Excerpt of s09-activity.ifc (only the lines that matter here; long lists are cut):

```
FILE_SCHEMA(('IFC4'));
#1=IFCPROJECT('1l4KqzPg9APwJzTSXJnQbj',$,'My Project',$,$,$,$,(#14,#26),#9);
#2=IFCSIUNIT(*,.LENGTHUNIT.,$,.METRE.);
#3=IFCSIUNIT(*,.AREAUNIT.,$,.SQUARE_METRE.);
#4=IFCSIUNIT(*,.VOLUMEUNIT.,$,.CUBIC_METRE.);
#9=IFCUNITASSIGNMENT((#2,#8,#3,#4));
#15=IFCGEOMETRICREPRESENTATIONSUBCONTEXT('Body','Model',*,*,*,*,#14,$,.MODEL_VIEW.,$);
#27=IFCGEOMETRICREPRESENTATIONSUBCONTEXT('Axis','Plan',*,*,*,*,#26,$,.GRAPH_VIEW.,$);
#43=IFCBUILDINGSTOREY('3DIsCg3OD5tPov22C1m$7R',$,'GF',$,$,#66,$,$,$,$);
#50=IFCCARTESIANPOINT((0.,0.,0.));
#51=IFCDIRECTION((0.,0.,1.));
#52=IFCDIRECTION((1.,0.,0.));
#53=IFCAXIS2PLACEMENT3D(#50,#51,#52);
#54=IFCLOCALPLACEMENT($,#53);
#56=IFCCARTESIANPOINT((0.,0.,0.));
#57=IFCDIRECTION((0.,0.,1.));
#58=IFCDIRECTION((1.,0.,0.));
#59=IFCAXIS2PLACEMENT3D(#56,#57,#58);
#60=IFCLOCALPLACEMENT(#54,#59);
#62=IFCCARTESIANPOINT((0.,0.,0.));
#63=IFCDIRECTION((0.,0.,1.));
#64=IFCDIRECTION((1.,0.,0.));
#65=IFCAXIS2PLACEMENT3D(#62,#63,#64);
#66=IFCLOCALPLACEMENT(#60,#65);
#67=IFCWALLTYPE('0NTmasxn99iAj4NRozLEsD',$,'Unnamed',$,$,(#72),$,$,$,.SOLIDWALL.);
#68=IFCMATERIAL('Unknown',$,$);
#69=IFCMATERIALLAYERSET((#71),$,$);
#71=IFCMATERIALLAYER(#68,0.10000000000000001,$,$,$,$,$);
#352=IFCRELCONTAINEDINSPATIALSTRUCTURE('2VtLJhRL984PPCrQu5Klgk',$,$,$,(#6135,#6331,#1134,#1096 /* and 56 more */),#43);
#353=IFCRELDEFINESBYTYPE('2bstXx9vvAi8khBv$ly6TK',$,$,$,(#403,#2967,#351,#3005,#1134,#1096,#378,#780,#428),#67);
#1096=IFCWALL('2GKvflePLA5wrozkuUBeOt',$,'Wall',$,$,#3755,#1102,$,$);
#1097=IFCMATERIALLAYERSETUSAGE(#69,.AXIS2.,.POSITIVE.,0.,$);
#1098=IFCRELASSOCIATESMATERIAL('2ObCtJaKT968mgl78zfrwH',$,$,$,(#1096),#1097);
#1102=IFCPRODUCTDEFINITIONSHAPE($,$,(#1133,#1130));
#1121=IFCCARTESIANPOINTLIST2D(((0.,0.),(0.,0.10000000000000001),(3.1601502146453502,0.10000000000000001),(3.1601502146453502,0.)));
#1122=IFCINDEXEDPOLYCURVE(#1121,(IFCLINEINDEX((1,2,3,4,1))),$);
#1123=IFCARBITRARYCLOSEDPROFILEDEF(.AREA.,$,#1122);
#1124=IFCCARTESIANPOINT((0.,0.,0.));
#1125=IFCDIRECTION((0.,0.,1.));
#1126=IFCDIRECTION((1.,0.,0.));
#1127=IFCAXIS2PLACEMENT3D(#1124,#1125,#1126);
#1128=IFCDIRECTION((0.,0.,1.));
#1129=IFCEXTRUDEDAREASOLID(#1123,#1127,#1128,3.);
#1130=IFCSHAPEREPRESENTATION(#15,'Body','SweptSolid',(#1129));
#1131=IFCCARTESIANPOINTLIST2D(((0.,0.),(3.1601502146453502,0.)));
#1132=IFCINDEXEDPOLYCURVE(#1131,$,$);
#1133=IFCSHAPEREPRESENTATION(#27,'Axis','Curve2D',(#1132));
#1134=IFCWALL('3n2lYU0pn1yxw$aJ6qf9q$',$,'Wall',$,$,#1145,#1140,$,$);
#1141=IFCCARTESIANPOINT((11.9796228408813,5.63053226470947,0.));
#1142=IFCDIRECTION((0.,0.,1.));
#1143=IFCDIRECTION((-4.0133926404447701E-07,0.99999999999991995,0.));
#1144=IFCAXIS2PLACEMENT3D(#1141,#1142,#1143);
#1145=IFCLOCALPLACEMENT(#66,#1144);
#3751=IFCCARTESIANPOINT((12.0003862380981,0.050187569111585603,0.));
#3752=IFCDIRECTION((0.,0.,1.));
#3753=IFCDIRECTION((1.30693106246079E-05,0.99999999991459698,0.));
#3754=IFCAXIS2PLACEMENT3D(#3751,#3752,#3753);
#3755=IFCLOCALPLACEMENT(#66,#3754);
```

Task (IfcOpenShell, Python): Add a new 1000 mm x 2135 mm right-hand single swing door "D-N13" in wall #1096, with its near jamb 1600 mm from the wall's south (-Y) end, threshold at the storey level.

```python
import numpy as np
import ifcopenshell
import ifcopenshell.api.feature
import ifcopenshell.api.geometry
import ifcopenshell.api.root
import ifcopenshell.api.spatial
import ifcopenshell.geom
import ifcopenshell.util.element
import ifcopenshell.util.placement
import ifcopenshell.util.representation
import ifcopenshell.util.shape
import ifcopenshell.util.unit

model = ifcopenshell.open("s09-activity.ifc")
unit_scale = ifcopenshell.util.unit.calculate_unit_scale(model)
settings = ifcopenshell.geom.settings()


def volume(element):
    """Net volume in cubic metres, openings subtracted."""
    shape = ifcopenshell.geom.create_shape(settings, element)
    return ifcopenshell.util.shape.get_volume(shape.geometry)


wall = model.by_guid("2GKvflePLA5wrozkuUBeOt")
storey = ifcopenshell.util.element.get_container(wall, ifc_class="IfcBuildingStorey")
context = ifcopenshell.util.representation.get_context(model, "Model", "Body", "MODEL_VIEW")
before = volume(wall)

width, height, from_end, sill = 1, 2.135, 1.6, 0.0  # metres

# The wall runs along its own X axis, and the end named is its -X end.
wall_shape = ifcopenshell.geom.create_shape(settings, wall)
x, y, z = ifcopenshell.util.shape.get_vertices(wall_shape.geometry).T
start = x.min() + from_end
face, thickness = float(y.min()), float(y.max() - y.min())
wall_matrix = ifcopenshell.util.placement.get_local_placement(wall.ObjectPlacement)
level = ifcopenshell.util.placement.get_local_placement(storey.ObjectPlacement)[2, 3]


def in_wall(x, y):
    """Placement at x, y metres in the wall's axes, at sill height."""
    matrix = wall_matrix.copy()
    matrix[:, 3] = wall_matrix @ np.array([x / unit_scale, y / unit_scale, 0.0, 1.0])
    matrix[2, 3] = level + sill / unit_scale
    return matrix


# Opening: a box that overshoots both wall faces by 50 mm.
opening = ifcopenshell.api.root.create_entity(model, ifc_class="IfcOpeningElement", predefined_type="OPENING")
box = ifcopenshell.api.geometry.add_wall_representation(
    model, context=context, length=width, height=height, thickness=thickness + 0.1
)
ifcopenshell.api.geometry.assign_representation(model, product=opening, representation=box)
ifcopenshell.api.geometry.edit_object_placement(model, product=opening, matrix=in_wall(start, face - 0.05), is_si=False)
ifcopenshell.api.feature.add_feature(model, feature=opening, element=wall)

door = ifcopenshell.api.root.create_entity(model, ifc_class="IfcDoor", name="D-N13", predefined_type="DOOR")
door.OverallWidth, door.OverallHeight = width / unit_scale, height / unit_scale
door.OperationType = "SINGLE_SWING_RIGHT"
body = ifcopenshell.api.geometry.add_door_representation(
    model,
    context=context,
    overall_width=door.OverallWidth,
    overall_height=door.OverallHeight,
    operation_type="SINGLE_SWING_RIGHT",
    lining_properties={"LiningDepth": thickness / unit_scale, "ThresholdDepth": thickness / unit_scale},
)
ifcopenshell.api.geometry.assign_representation(model, product=door, representation=body)
ifcopenshell.api.spatial.assign_container(model, products=[door], relating_structure=storey)
ifcopenshell.api.feature.add_filling(model, opening=opening, element=door)

# The lining spans the wall, so the door starts at the wall face.
ifcopenshell.api.geometry.edit_object_placement(model, product=door, matrix=in_wall(start, face), is_si=False)

after = volume(wall)

print(f"wall volume {before:.3f} -> {after:.3f} m3")

model.write("s09-activity-out.ifc")
```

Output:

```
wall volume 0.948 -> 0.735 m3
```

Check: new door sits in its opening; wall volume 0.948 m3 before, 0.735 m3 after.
